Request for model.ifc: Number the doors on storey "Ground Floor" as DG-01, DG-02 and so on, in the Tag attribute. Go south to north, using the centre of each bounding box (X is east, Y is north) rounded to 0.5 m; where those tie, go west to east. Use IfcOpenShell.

First a look at what the model holds.

```python
import ifcopenshell
import ifcopenshell.util.element
import ifcopenshell.util.placement

model = ifcopenshell.open("model.ifc")
print(model.schema)
storey = next(s for s in model.by_type("IfcBuildingStorey") if s.Name == "Ground Floor")
doors = [e for e in ifcopenshell.util.element.get_decomposition(storey) if e.is_a("IfcDoor")]
for e in sorted(doors, key=lambda e: e.id()):
    origin = ifcopenshell.util.placement.get_local_placement(e.ObjectPlacement)[:3, 3]
    print(e.id(), e.Tag, e.Name, origin.round(2) + 0.0, sep=" | ")
```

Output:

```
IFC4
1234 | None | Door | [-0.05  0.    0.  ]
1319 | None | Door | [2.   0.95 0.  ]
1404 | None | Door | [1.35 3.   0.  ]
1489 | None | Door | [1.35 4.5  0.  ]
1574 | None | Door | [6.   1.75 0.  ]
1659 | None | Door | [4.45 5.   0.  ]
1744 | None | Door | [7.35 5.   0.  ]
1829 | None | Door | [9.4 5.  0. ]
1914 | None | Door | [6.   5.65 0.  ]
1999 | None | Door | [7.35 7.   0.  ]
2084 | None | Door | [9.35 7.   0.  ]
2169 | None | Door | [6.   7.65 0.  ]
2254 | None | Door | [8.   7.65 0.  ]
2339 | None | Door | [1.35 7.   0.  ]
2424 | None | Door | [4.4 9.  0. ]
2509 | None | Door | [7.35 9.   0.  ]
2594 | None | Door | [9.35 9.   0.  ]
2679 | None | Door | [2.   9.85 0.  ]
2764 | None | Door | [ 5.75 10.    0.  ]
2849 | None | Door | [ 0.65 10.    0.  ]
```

```python
import ifcopenshell
import ifcopenshell.geom
import ifcopenshell.util.element
import ifcopenshell.util.shape

model = ifcopenshell.open("model.ifc")
settings = ifcopenshell.geom.settings()
settings.set("use-world-coords", True)


def centre(element):
    shape = ifcopenshell.geom.create_shape(settings, element)
    return ifcopenshell.util.shape.get_bbox_centroid(shape.geometry)


storey = next(s for s in model.by_type("IfcBuildingStorey") if s.Name == "Ground Floor")
doors = [e for e in ifcopenshell.util.element.get_decomposition(storey) if e.is_a("IfcDoor")]

# Insertion points can sit at a corner or the storey origin, so sort by the geometry (in metres).
centres = {e: centre(e) for e in doors}
doors.sort(key=lambda e: (round(centres[e][1] / 0.5), centres[e][0]))

for i, e in enumerate(doors, start=1):
    number = f"DG-{i:02d}"
    e.Tag = number
    print(e.id(), number)

model.write("model-out.ifc")
```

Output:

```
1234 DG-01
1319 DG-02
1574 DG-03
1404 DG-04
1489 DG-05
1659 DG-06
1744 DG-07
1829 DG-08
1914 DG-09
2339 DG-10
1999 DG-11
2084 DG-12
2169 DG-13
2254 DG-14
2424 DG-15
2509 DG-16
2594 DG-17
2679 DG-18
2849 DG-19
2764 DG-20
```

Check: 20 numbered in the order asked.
